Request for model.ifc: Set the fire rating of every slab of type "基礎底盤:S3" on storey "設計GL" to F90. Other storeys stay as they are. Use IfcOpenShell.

First a look at what the model holds.

```python
import ifcopenshell
import ifcopenshell.util.element

model = ifcopenshell.open("model.ifc")
print(model.schema)
storey = next(s for s in model.by_type("IfcBuildingStorey") if s.Name == "設計GL")
slabs = [e for e in ifcopenshell.util.element.get_decomposition(storey) if e.is_a("IfcSlab")]
seen = {}
for e in slabs:
    element_type = ifcopenshell.util.element.get_type(e)
    key = (element_type.Name if element_type != e and element_type else None, ifcopenshell.util.element.get_pset(e, "Pset_SlabCommon", "FireRating"))
    seen[key] = seen.get(key, 0) + 1
for (name, value), count in sorted(seen.items(), key=str):
    print(count, "x", name, "|", value)
```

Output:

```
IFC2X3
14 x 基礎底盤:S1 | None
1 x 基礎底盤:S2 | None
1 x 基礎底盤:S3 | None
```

```python
import ifcopenshell
import ifcopenshell.api.pset
import ifcopenshell.util.element

model = ifcopenshell.open("model.ifc")

storey = next(s for s in model.by_type("IfcBuildingStorey") if s.Name == "設計GL")
slabs = [e for e in ifcopenshell.util.element.get_decomposition(storey) if e.is_a("IfcSlab")]

count = 0
for e in slabs:
    element_type = ifcopenshell.util.element.get_type(e)
    if element_type in (None, e) or element_type.Name != "基礎底盤:S3":
        continue
    # add_pset returns the element's existing set when there is one.
    pset = ifcopenshell.api.pset.add_pset(model, product=e, name="Pset_SlabCommon")
    ifcopenshell.api.pset.edit_pset(model, pset=pset, properties={"FireRating": "F90"})
    count += 1

print(count, "slabs updated")

model.write("model_v2.ifc")
```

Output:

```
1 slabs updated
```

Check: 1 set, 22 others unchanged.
